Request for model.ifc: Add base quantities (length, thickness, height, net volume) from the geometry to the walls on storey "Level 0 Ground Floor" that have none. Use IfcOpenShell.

First a look at what the model holds.

```python
import ifcopenshell
import ifcopenshell.util.element
import ifcopenshell.util.unit

model = ifcopenshell.open("model.ifc")
print(model.schema)
for unit_type in ("LENGTHUNIT", "AREAUNIT", "VOLUMEUNIT"):
    print(unit_type, ifcopenshell.util.unit.calculate_unit_scale(model, unit_type))
storey = next(s for s in model.by_type("IfcBuildingStorey") if s.Name == "Level 0 Ground Floor")
walls = [e for e in ifcopenshell.util.element.get_decomposition(storey) if e.is_a("IfcWall")]
for e in sorted(walls, key=lambda e: e.id()):
    print(e.id(), e.is_a(), e.Name, list(ifcopenshell.util.element.get_psets(e, qtos_only=True)), sep=" | ")
```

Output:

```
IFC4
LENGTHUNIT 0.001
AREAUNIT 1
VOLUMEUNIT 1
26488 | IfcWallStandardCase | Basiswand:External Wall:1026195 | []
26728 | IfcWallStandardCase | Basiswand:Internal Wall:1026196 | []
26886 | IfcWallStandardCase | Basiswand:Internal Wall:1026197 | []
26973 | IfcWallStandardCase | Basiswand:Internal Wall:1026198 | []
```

```python
import ifcopenshell
import ifcopenshell.api.pset
import ifcopenshell.geom
import ifcopenshell.util.element
import ifcopenshell.util.shape
import ifcopenshell.util.unit

model = ifcopenshell.open("model.ifc")
unit_scale = ifcopenshell.util.unit.calculate_unit_scale(model)
volume_scale = ifcopenshell.util.unit.calculate_unit_scale(model, "VOLUMEUNIT")
settings = ifcopenshell.geom.settings()

storey = next(s for s in model.by_type("IfcBuildingStorey") if s.Name == "Level 0 Ground Floor")
walls = [e for e in ifcopenshell.util.element.get_decomposition(storey) if e.is_a("IfcWall")]

for e in sorted(walls, key=lambda e: e.id()):
    if ifcopenshell.util.element.get_psets(e, qtos_only=True, should_inherit=False):
        continue
    # Geometry comes back in metres, in the element's own axes.
    shape = ifcopenshell.geom.create_shape(settings, e)
    values = {
        "Length": ifcopenshell.util.shape.get_x(shape.geometry) / unit_scale,
        "Width": ifcopenshell.util.shape.get_y(shape.geometry) / unit_scale,
        "Height": ifcopenshell.util.shape.get_z(shape.geometry) / unit_scale,
        "NetVolume": ifcopenshell.util.shape.get_volume(shape.geometry) / volume_scale,
    }
    qto = ifcopenshell.api.pset.add_qto(model, product=e, name="Qto_WallBaseQuantities")
    ifcopenshell.api.pset.edit_qto(model, qto=qto, properties=values)
    print(e.id(), {k: round(v, 3) for k, v in values.items()})

model.write("model_edited.ifc")
```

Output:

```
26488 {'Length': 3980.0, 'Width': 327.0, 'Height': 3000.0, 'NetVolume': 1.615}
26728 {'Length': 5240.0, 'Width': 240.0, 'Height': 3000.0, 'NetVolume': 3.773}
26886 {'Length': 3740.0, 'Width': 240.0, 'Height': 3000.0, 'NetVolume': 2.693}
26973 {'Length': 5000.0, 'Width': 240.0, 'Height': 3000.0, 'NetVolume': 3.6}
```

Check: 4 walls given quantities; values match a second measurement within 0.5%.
